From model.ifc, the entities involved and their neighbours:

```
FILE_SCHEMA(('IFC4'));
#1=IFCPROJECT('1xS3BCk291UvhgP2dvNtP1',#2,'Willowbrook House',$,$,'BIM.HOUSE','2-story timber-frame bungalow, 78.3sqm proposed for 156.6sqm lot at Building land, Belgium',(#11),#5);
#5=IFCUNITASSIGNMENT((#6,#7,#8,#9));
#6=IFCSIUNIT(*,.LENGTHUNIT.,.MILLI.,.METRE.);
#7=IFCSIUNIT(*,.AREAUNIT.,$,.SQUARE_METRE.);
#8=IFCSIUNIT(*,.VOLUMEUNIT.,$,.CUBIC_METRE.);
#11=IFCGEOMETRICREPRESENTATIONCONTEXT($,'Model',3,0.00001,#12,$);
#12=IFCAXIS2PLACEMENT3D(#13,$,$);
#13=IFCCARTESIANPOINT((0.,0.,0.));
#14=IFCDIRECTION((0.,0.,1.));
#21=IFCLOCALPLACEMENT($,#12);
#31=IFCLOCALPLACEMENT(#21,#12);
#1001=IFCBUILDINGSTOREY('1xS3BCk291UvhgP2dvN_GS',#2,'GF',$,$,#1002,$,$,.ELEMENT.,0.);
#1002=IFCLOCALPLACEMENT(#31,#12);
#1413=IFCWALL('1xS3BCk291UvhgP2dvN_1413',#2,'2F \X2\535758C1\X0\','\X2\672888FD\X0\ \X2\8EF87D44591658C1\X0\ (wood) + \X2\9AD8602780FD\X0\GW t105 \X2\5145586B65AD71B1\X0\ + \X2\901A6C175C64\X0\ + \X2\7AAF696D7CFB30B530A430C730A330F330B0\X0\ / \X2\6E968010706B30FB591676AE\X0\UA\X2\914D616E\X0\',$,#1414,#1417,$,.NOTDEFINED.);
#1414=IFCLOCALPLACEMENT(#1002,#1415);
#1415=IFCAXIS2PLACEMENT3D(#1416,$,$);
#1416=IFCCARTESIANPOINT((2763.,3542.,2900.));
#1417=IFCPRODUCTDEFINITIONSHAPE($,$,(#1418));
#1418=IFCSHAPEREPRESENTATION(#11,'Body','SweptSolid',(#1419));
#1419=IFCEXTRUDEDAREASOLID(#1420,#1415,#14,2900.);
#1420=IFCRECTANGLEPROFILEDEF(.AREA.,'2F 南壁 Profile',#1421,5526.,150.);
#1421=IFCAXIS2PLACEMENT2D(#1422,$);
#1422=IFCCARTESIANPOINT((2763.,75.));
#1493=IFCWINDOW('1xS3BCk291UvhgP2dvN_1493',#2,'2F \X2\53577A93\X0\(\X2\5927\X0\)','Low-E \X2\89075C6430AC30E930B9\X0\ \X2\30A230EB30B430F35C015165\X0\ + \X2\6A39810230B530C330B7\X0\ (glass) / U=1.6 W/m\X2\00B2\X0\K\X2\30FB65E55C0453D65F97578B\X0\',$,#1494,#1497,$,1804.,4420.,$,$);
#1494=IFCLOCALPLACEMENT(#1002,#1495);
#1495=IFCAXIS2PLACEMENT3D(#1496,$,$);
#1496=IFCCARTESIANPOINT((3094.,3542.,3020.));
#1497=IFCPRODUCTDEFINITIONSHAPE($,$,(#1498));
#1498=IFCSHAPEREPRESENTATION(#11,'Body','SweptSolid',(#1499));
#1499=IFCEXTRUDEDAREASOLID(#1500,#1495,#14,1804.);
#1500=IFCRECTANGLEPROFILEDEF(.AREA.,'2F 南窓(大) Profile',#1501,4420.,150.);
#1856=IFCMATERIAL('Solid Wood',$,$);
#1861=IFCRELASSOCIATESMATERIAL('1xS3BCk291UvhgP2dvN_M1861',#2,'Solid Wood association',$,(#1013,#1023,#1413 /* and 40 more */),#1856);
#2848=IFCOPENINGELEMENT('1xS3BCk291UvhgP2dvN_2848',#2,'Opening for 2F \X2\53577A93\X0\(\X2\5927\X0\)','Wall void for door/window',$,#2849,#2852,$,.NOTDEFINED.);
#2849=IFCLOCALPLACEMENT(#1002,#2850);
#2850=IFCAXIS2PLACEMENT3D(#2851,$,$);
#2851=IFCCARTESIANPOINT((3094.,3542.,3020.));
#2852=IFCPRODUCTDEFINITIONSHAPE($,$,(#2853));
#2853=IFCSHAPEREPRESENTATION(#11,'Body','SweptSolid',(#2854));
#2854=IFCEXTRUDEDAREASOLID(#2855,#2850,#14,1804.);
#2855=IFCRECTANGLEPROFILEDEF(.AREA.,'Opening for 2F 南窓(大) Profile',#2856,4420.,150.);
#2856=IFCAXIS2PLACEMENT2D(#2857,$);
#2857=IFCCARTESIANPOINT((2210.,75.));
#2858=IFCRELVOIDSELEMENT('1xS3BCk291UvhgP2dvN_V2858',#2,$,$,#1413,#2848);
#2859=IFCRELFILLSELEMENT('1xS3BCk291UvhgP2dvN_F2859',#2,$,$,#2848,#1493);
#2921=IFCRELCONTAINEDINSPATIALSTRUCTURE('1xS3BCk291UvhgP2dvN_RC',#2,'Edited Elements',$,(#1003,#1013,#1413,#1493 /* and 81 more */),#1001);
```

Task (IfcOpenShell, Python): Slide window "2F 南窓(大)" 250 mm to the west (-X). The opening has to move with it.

```python
import ifcopenshell
import ifcopenshell.api.geometry
import ifcopenshell.util.placement
import ifcopenshell.util.unit

model = ifcopenshell.open("model.ifc")
unit_scale = ifcopenshell.util.unit.calculate_unit_scale(model)

window = model.by_guid("1xS3BCk291UvhgP2dvN_1493")
opening = window.FillsVoids[0].RelatingOpeningElement
wall = opening.VoidsElements[0].RelatingBuildingElement

wall_matrix = ifcopenshell.util.placement.get_local_placement(wall.ObjectPlacement)
shift = wall_matrix[:3, 0] * -0.25 / unit_scale
before = ifcopenshell.util.placement.get_local_placement(window.ObjectPlacement)[:3, 3].copy()

# The window is not placed relative to its opening, so move both.
for product in (opening, window):
    matrix = ifcopenshell.util.placement.get_local_placement(product.ObjectPlacement)
    matrix[:3, 3] += shift
    ifcopenshell.api.geometry.edit_object_placement(model, product=product, matrix=matrix, is_si=False)

after = ifcopenshell.util.placement.get_local_placement(window.ObjectPlacement)[:3, 3]
print("window moved by", (after - before).round(3) + 0.0)

model.write("model-out.ifc")
```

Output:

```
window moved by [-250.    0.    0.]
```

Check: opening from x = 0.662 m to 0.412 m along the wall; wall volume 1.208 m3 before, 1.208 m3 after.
